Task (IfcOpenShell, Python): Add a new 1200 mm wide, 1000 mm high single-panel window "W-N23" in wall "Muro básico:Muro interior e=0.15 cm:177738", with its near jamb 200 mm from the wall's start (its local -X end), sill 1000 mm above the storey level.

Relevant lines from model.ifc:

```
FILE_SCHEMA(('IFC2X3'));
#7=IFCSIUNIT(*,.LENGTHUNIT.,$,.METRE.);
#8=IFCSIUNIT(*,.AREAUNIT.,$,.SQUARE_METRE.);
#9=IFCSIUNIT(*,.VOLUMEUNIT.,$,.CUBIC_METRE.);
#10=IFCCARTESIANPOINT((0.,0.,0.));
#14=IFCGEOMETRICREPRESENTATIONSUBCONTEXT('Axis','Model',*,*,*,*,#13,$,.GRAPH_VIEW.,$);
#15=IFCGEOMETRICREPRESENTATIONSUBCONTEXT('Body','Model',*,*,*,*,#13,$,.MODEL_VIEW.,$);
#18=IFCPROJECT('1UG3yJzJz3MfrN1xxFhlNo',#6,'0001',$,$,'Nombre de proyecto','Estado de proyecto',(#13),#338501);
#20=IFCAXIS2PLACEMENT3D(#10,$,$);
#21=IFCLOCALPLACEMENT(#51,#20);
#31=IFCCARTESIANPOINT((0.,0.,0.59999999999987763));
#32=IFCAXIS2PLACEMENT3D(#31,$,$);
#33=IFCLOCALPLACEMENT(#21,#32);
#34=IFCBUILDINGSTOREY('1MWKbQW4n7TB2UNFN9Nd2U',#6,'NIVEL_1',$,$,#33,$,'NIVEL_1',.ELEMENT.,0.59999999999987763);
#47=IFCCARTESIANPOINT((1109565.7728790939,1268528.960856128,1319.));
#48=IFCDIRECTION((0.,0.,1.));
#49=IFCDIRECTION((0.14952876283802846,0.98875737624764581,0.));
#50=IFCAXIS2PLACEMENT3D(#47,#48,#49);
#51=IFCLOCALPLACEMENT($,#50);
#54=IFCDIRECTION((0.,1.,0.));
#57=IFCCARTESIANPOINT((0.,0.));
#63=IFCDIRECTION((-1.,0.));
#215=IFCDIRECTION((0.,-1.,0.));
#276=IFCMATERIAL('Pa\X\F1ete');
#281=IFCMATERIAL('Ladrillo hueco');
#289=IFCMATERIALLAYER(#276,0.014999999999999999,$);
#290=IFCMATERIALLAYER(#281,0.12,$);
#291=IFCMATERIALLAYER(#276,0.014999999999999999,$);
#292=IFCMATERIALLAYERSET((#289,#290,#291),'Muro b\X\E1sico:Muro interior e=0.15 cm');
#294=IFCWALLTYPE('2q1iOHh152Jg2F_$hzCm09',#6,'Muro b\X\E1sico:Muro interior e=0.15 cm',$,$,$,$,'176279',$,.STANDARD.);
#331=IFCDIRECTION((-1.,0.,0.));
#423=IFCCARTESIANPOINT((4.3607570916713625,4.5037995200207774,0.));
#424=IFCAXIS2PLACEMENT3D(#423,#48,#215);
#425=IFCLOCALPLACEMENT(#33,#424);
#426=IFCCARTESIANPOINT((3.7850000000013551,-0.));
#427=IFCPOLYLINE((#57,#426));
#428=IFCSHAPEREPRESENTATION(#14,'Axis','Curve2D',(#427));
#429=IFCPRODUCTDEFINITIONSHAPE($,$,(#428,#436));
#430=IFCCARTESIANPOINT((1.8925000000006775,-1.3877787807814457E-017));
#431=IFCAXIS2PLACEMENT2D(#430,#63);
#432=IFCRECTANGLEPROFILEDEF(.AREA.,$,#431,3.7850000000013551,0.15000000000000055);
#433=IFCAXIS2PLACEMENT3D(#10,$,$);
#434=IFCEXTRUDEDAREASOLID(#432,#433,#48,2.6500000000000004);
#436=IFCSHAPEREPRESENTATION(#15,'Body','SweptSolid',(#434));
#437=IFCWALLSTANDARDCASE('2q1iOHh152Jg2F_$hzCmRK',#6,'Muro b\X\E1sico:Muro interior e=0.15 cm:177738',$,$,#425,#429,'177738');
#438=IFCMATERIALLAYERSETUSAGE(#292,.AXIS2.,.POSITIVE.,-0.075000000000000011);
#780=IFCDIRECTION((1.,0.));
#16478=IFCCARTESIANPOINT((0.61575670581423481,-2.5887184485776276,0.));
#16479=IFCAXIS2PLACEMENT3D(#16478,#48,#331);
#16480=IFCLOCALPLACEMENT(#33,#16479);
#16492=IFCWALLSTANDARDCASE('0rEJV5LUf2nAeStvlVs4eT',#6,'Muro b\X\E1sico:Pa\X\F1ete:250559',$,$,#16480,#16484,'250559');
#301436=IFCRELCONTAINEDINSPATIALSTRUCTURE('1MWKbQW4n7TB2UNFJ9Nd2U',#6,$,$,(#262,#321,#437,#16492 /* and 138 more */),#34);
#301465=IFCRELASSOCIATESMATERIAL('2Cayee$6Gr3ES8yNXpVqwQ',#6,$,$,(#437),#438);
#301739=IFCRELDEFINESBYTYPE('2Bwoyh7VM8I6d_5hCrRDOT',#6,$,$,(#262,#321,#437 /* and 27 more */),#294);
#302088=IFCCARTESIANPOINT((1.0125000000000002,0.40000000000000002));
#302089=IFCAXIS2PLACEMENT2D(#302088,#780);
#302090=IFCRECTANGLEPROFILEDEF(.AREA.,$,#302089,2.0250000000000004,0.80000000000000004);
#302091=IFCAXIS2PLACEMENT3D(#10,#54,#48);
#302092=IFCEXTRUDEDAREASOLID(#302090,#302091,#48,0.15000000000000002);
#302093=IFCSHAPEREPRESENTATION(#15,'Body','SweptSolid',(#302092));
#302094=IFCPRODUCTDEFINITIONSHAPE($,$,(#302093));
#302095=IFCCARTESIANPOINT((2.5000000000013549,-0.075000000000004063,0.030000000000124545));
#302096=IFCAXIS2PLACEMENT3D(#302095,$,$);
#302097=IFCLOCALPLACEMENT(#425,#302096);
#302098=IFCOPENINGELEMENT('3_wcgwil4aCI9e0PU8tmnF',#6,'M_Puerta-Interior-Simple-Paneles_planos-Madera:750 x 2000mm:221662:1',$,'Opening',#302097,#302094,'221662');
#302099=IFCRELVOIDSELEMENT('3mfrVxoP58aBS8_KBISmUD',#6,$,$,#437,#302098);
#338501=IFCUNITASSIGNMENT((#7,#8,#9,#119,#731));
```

```python
import numpy as np
import ifcopenshell
import ifcopenshell.api.feature
import ifcopenshell.api.geometry
import ifcopenshell.api.root
import ifcopenshell.api.spatial
import ifcopenshell.api.type
import ifcopenshell.geom
import ifcopenshell.util.element
import ifcopenshell.util.placement
import ifcopenshell.util.representation
import ifcopenshell.util.shape
import ifcopenshell.util.unit

model = ifcopenshell.open("model.ifc")
unit_scale = ifcopenshell.util.unit.calculate_unit_scale(model)
settings = ifcopenshell.geom.settings()


def volume(element):
    """Net volume in cubic metres, openings subtracted."""
    shape = ifcopenshell.geom.create_shape(settings, element)
    return ifcopenshell.util.shape.get_volume(shape.geometry)


wall = model.by_id(437)
storey = ifcopenshell.util.element.get_container(wall, ifc_class="IfcBuildingStorey")
context = ifcopenshell.util.representation.get_context(model, "Model", "Body", "MODEL_VIEW")
before = volume(wall)

width, height, from_end, sill = 1.2, 1, 0.2, 1  # metres

# The wall runs along its own X axis, and the end named is its -X end.
wall_shape = ifcopenshell.geom.create_shape(settings, wall)
x, y, z = ifcopenshell.util.shape.get_vertices(wall_shape.geometry).T
start = x.min() + from_end
face, thickness = float(y.min()), float(y.max() - y.min())
wall_matrix = ifcopenshell.util.placement.get_local_placement(wall.ObjectPlacement)
level = ifcopenshell.util.placement.get_local_placement(storey.ObjectPlacement)[2, 3]


def in_wall(x, y):
    """Placement at x, y metres in the wall's axes, at sill height."""
    matrix = wall_matrix.copy()
    matrix[:, 3] = wall_matrix @ np.array([x / unit_scale, y / unit_scale, 0.0, 1.0])
    matrix[2, 3] = level + sill / unit_scale
    return matrix


# Opening: a box that overshoots both wall faces by 50 mm.
opening = ifcopenshell.api.root.create_entity(model, ifc_class="IfcOpeningElement")
box = ifcopenshell.api.geometry.add_wall_representation(
    model, context=context, length=width, height=height, thickness=thickness + 0.1
)
ifcopenshell.api.geometry.assign_representation(model, product=opening, representation=box)
ifcopenshell.api.geometry.edit_object_placement(model, product=opening, matrix=in_wall(start, face - 0.05), is_si=False)
ifcopenshell.api.feature.add_feature(model, feature=opening, element=wall)

window = ifcopenshell.api.root.create_entity(model, ifc_class="IfcWindow", name="W-N23")
window.OverallWidth, window.OverallHeight = width / unit_scale, height / unit_scale
body = ifcopenshell.api.geometry.add_window_representation(
    model,
    context=context,
    overall_width=window.OverallWidth,
    overall_height=window.OverallHeight,
    partition_type="SINGLE_PANEL",
)
ifcopenshell.api.geometry.assign_representation(model, product=window, representation=body)
ifcopenshell.api.spatial.assign_container(model, products=[window], relating_structure=storey)
fills = ifcopenshell.api.feature.add_filling(model, opening=opening, element=window)
fills.OwnerHistory = window.OwnerHistory  # required in IFC2X3

# IFC2X3 keeps the operation on the window style.
style = ifcopenshell.api.root.create_entity(model, ifc_class="IfcWindowStyle", name="W-N23")
style.OperationType, style.ConstructionType = "SINGLE_PANEL", "NOTDEFINED"
style.ParameterTakesPrecedence = style.Sizeable = False
ifcopenshell.api.type.assign_type(model, related_objects=[window], relating_type=style)

# Centre the window in the wall's thickness.
ifcopenshell.api.geometry.edit_object_placement(model, product=window, matrix=in_wall(start, face), is_si=False)
window_shape = ifcopenshell.geom.create_shape(settings, window)
depth = ifcopenshell.util.shape.get_vertices(window_shape.geometry)[:, 1]
offset = face + thickness / 2 - (depth.min() + depth.max()) / 2
ifcopenshell.api.geometry.edit_object_placement(model, product=window, matrix=in_wall(start, offset), is_si=False)

after = volume(wall)

print(f"wall volume {before:.3f} -> {after:.3f} m3")

model.write("model_updated.ifc")
```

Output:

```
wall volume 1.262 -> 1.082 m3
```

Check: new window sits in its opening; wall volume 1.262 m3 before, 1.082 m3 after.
